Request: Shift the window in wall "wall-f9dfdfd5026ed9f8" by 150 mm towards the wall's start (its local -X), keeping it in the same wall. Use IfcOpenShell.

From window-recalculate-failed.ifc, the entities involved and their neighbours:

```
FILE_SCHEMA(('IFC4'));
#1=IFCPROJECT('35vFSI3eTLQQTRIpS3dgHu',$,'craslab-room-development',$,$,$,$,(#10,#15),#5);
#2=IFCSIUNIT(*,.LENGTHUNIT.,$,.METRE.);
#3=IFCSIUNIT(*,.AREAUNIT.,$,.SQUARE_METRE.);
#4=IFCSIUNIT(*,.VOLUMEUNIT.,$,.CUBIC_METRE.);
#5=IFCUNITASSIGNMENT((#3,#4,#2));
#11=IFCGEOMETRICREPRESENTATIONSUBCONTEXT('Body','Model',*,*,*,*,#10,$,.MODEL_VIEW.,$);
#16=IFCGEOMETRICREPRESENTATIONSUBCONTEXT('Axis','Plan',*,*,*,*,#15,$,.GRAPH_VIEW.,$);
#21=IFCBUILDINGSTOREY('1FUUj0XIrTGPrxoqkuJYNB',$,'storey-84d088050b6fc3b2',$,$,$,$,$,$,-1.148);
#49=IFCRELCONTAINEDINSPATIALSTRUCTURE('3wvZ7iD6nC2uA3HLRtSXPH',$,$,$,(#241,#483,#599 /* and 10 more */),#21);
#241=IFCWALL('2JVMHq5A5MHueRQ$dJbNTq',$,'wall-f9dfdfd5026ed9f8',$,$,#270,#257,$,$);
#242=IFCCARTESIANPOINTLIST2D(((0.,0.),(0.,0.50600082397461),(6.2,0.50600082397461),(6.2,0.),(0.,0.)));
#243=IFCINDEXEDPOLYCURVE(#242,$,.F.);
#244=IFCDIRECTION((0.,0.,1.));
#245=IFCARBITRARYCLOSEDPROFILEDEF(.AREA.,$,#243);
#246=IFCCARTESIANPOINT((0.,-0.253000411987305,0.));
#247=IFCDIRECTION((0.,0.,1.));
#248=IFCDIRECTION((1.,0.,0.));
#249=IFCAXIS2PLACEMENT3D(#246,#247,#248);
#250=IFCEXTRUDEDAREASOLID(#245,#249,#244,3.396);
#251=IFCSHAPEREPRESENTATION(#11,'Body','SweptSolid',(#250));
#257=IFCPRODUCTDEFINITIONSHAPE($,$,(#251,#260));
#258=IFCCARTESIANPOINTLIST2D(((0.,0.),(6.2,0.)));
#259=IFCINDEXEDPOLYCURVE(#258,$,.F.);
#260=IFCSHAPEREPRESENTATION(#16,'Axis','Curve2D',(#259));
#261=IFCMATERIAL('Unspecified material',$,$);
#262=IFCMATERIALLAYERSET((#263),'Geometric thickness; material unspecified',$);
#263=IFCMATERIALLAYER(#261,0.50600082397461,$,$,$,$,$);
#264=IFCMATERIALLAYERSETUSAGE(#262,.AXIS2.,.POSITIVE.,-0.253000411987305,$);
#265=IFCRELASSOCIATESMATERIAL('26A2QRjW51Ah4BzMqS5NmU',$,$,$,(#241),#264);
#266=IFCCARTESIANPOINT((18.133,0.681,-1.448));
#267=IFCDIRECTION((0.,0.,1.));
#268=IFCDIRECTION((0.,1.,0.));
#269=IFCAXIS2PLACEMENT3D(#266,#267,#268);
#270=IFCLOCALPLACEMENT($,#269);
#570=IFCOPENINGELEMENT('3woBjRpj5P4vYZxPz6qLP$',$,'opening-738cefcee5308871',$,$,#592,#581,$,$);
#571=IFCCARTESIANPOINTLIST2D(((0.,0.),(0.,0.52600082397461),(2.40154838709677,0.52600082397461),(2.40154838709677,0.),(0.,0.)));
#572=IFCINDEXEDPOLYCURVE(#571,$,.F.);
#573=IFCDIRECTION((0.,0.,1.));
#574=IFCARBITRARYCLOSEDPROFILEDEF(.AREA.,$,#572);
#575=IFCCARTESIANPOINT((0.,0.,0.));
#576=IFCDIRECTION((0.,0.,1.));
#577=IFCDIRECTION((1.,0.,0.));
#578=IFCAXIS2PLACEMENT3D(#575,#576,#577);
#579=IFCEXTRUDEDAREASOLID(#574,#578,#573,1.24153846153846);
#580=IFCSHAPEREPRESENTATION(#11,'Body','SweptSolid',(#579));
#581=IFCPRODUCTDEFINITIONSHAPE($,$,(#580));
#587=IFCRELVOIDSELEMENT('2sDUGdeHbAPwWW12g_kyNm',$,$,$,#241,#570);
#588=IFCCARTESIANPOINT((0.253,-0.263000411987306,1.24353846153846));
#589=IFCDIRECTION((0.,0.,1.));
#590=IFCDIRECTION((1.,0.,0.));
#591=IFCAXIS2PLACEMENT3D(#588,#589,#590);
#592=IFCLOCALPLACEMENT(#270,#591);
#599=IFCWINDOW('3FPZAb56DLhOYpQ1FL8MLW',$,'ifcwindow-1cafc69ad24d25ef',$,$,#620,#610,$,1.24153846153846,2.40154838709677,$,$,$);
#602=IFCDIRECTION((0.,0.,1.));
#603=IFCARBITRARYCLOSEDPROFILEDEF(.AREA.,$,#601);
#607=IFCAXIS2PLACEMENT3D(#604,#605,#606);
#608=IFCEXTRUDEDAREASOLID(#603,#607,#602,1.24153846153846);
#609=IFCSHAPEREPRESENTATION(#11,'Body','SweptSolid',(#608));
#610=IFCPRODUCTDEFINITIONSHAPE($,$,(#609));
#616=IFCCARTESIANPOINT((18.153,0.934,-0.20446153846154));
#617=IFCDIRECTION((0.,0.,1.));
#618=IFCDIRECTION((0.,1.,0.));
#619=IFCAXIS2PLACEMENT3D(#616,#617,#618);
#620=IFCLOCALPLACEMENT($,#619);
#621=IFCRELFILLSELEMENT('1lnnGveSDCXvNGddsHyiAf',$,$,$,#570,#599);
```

```python
import ifcopenshell
import ifcopenshell.api.geometry
import ifcopenshell.util.placement

model = ifcopenshell.open("window-recalculate-failed.ifc")

window = model.by_guid("3FPZAb56DLhOYpQ1FL8MLW")
opening = window.FillsVoids[0].RelatingOpeningElement
wall = opening.VoidsElements[0].RelatingBuildingElement

wall_matrix = ifcopenshell.util.placement.get_local_placement(wall.ObjectPlacement)
shift = wall_matrix[:3, 0] * -0.15
before = ifcopenshell.util.placement.get_local_placement(window.ObjectPlacement)[:3, 3].copy()

# The window is not placed relative to its opening, so move both.
for product in (opening, window):
    matrix = ifcopenshell.util.placement.get_local_placement(product.ObjectPlacement)
    matrix[:3, 3] += shift
    ifcopenshell.api.geometry.edit_object_placement(model, product=product, matrix=matrix, is_si=False)

after = ifcopenshell.util.placement.get_local_placement(window.ObjectPlacement)[:3, 3]
print("window moved by", (after - before).round(3) + 0.0)

model.write("window-recalculate-failed_rev.ifc")
```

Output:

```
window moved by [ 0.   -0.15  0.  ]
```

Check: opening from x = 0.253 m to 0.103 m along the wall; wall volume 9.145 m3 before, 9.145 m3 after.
